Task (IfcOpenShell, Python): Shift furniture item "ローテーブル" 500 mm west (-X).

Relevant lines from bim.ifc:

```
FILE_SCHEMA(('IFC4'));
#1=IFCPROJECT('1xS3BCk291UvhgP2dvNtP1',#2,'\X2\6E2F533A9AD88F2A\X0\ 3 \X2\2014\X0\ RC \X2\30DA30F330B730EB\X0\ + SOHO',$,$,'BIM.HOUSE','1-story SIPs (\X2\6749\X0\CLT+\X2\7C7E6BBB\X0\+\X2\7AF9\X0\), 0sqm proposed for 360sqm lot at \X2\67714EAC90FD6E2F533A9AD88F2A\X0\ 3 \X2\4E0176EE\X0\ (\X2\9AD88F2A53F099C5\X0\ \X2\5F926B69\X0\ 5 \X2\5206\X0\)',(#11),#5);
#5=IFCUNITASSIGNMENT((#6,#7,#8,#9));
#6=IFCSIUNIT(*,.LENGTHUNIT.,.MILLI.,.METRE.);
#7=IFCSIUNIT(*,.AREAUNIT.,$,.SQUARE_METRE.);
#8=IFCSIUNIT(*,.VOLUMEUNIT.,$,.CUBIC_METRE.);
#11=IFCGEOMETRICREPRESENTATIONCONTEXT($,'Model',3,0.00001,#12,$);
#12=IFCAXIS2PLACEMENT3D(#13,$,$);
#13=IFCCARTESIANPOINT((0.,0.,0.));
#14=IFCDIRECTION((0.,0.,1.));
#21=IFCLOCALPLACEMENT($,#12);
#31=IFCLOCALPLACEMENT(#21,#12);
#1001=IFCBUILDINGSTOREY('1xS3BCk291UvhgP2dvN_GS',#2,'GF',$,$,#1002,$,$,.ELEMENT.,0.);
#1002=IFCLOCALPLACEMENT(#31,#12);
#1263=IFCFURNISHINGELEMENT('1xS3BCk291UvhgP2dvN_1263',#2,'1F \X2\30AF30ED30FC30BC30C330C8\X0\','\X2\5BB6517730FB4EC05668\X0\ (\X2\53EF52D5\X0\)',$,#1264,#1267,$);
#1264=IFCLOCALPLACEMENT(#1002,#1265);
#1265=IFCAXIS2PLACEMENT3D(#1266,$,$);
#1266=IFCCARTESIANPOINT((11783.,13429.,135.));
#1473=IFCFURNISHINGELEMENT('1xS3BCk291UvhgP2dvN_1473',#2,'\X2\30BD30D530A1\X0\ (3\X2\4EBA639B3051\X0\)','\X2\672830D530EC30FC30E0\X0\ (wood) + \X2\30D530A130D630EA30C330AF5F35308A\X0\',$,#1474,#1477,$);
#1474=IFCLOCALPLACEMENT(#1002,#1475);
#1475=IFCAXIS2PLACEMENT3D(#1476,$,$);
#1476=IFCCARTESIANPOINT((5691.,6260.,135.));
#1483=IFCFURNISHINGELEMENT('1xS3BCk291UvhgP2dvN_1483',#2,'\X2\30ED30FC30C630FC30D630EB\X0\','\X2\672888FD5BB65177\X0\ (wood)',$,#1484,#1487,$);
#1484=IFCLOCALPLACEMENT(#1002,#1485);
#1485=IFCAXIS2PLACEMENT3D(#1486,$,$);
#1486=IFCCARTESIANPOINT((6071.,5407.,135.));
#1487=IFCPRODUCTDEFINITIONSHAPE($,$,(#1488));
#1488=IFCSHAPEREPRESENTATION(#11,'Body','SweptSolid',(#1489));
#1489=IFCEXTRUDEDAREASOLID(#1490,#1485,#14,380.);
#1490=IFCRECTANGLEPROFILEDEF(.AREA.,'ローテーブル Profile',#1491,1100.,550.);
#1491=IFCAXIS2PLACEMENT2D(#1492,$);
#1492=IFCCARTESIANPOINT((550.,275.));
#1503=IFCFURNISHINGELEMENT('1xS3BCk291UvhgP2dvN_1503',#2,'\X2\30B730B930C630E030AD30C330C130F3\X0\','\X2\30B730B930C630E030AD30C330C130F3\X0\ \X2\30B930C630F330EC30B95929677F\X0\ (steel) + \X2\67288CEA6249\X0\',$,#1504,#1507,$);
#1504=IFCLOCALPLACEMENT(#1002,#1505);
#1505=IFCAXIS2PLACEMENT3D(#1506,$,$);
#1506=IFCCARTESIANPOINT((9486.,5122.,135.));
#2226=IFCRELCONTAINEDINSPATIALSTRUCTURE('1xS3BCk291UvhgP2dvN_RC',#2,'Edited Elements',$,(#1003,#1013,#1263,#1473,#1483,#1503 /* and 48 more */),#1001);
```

```python
import ifcopenshell
import ifcopenshell.api.geometry
import ifcopenshell.util.placement
import ifcopenshell.util.unit

model = ifcopenshell.open("bim.ifc")
unit_scale = ifcopenshell.util.unit.calculate_unit_scale(model)

item = model.by_guid("1xS3BCk291UvhgP2dvN_1483")
matrix = ifcopenshell.util.placement.get_local_placement(item.ObjectPlacement)
matrix[0, 3] -= 0.5 / unit_scale
ifcopenshell.api.geometry.edit_object_placement(model, product=item, matrix=matrix, is_si=False)

print(ifcopenshell.util.placement.get_local_placement(item.ObjectPlacement).round(3) + 0.0)

model.write("bim_v2.ifc")
```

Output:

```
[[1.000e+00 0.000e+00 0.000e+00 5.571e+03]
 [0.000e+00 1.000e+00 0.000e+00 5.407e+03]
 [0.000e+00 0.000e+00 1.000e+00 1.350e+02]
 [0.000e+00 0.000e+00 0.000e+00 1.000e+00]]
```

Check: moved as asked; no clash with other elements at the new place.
